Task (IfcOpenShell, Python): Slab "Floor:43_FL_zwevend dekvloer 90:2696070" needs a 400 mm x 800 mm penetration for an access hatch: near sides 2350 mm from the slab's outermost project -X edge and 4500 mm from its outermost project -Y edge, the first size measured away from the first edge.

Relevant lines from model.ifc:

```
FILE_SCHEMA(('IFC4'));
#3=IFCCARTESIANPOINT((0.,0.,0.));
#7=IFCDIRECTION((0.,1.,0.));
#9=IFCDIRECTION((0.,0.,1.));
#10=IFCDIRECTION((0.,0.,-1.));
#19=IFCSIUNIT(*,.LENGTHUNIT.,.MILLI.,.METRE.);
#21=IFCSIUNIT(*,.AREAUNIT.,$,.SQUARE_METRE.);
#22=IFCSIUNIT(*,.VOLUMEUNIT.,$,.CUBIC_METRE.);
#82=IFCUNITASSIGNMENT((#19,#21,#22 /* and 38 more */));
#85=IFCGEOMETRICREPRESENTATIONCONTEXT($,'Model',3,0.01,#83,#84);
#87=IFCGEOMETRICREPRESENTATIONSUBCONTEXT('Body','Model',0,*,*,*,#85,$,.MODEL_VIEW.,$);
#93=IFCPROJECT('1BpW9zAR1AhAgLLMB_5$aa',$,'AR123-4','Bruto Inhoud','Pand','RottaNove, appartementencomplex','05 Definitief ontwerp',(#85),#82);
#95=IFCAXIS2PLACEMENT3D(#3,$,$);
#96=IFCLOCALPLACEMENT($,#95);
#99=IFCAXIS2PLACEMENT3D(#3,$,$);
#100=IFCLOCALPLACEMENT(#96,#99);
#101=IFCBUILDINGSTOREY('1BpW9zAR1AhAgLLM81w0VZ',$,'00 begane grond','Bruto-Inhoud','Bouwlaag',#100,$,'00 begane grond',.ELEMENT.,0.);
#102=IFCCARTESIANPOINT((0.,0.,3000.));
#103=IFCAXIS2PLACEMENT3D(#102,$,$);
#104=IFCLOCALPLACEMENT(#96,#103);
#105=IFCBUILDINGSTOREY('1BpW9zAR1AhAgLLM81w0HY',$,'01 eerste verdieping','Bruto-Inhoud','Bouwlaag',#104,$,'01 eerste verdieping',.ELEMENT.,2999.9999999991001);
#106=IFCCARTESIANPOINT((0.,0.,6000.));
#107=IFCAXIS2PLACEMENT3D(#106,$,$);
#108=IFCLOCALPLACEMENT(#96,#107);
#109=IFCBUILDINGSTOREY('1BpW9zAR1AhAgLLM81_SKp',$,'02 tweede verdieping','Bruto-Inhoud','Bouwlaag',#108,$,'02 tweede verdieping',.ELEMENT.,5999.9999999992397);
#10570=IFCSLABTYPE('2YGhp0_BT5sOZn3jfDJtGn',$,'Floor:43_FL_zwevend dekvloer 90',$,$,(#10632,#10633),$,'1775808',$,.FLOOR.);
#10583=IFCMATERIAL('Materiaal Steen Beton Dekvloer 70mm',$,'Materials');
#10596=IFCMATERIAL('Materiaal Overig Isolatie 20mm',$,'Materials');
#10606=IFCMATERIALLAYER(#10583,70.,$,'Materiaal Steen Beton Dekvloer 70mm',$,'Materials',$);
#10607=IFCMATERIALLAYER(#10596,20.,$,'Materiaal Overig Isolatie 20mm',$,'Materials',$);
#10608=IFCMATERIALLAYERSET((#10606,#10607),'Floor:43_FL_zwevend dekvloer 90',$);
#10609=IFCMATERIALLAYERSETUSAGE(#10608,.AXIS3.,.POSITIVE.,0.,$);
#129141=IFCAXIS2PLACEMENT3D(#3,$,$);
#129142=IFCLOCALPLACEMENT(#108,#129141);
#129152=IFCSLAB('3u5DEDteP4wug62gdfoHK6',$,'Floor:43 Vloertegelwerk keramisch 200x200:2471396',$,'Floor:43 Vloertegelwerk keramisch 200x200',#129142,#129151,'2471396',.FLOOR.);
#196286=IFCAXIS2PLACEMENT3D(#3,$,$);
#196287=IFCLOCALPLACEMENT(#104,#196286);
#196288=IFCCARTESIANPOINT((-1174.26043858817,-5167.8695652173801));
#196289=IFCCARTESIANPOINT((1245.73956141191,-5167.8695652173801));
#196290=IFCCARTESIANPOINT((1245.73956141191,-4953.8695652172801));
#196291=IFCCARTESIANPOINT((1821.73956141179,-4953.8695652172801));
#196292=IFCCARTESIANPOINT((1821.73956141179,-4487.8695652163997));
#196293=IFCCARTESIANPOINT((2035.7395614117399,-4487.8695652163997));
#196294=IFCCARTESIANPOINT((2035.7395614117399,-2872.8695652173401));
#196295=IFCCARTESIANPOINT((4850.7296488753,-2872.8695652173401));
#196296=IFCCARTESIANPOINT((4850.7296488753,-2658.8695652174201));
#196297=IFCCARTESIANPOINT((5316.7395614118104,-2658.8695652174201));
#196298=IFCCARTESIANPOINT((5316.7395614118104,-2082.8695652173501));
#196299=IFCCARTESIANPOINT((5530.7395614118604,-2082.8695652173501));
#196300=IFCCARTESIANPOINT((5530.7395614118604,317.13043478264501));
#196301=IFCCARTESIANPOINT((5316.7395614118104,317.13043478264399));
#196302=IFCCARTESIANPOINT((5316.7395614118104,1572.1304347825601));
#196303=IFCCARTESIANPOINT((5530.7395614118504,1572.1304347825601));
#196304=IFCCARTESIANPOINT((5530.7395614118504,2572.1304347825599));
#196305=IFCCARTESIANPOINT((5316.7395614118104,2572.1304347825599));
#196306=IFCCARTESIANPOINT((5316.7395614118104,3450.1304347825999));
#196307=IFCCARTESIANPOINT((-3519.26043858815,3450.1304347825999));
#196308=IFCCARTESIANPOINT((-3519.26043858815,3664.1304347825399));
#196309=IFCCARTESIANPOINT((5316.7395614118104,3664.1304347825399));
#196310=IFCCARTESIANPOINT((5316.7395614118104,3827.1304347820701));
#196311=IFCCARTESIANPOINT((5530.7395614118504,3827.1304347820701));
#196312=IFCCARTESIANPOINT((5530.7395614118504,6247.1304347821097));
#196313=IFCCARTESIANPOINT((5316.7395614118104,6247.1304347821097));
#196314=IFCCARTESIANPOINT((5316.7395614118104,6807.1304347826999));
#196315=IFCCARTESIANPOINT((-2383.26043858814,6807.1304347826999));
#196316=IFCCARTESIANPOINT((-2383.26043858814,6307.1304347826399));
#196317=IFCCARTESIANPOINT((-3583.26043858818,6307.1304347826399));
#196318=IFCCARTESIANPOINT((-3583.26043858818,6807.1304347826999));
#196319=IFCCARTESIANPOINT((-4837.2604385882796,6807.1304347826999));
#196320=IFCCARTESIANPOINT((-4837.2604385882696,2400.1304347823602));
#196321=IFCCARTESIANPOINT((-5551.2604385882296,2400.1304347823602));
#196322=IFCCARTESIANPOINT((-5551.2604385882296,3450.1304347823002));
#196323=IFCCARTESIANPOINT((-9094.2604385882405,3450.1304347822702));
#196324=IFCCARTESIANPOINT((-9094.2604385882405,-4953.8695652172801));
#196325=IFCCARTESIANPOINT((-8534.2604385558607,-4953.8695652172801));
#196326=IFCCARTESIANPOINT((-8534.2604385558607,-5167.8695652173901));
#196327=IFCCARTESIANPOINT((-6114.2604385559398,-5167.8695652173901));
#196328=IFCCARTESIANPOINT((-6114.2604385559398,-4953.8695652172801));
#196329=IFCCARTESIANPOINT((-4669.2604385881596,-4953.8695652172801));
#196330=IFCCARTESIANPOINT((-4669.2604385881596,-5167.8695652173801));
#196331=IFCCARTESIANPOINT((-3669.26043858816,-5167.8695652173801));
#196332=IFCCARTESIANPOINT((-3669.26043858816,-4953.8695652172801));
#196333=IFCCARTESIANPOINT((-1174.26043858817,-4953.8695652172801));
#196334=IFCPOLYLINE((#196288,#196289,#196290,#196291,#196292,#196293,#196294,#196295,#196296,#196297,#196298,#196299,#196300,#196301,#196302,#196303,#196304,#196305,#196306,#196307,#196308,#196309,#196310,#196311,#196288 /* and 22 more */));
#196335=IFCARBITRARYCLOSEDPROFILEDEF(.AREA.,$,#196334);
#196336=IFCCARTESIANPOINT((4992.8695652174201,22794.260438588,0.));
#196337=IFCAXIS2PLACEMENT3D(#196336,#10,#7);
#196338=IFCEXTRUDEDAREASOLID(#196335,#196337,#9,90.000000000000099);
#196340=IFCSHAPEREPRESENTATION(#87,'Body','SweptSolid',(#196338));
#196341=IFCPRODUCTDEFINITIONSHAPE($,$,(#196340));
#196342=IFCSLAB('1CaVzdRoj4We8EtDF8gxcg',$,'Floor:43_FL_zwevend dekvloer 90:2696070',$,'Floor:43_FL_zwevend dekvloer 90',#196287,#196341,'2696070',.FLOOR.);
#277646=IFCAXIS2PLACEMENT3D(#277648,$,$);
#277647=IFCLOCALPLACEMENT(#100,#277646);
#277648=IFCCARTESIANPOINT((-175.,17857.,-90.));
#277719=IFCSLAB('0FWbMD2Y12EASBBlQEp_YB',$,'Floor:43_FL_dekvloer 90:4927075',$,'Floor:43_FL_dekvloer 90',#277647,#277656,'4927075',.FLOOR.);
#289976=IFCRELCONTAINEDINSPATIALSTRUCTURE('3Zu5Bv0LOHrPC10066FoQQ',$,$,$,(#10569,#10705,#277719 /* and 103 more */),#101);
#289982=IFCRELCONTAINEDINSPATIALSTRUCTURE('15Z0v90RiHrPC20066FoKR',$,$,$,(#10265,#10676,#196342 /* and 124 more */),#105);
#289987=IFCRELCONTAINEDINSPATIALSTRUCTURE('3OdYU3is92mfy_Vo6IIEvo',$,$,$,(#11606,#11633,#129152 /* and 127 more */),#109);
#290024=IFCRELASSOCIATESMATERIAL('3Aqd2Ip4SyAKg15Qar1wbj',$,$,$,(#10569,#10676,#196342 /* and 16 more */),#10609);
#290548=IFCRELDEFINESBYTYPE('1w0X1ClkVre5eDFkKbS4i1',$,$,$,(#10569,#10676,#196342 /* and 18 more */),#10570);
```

```python
import numpy as np
import ifcopenshell
import ifcopenshell.api.feature
import ifcopenshell.api.geometry
import ifcopenshell.api.root
import ifcopenshell.geom
import ifcopenshell.util.placement
import ifcopenshell.util.representation
import ifcopenshell.util.shape
import ifcopenshell.util.unit

model = ifcopenshell.open("model.ifc")
unit_scale = ifcopenshell.util.unit.calculate_unit_scale(model)
settings = ifcopenshell.geom.settings()


def volume(element):
    """Net volume in cubic metres, openings subtracted."""
    shape = ifcopenshell.geom.create_shape(settings, element)
    return ifcopenshell.util.shape.get_volume(shape.geometry)


slab = model.by_guid("1CaVzdRoj4We8EtDF8gxcg")
before = volume(slab)

# Extent in the slab's own axes, in metres. The edges named are its -X and -Y sides.
slab_shape = ifcopenshell.geom.create_shape(settings, slab)
vertices = ifcopenshell.util.shape.get_vertices(slab_shape.geometry)
x_min, y_min, bottom = vertices.min(axis=0)
top = vertices[:, 2].max()

opening = ifcopenshell.api.root.create_entity(model, ifc_class="IfcOpeningElement", name="Access hatch opening", predefined_type="OPENING")
context = ifcopenshell.util.representation.get_context(model, "Model", "Body", "MODEL_VIEW")
width, depth = 0.4, 0.8
outline = [(0.0, 0.0), (width, 0.0), (width, depth), (0.0, depth), (0.0, 0.0)]
# Overshoot both faces by 50 mm so the cut is clean.
shape = ifcopenshell.api.geometry.add_slab_representation(
    model, context=context, depth=top - bottom + 0.1, polyline=outline
)
ifcopenshell.api.geometry.assign_representation(model, product=opening, representation=shape)

matrix = ifcopenshell.util.placement.get_local_placement(slab.ObjectPlacement)
matrix[:, 3] = matrix @ np.append(np.array([x_min + 2.35, y_min + 4.5, bottom - 0.05]) / unit_scale, 1.0)
ifcopenshell.api.geometry.edit_object_placement(model, product=opening, matrix=matrix, is_si=False)
ifcopenshell.api.feature.add_feature(model, feature=opening, element=slab)

after = volume(slab)

print(f"slab volume {before:.3f} -> {after:.3f} m3")

model.write("model-out.ifc")
```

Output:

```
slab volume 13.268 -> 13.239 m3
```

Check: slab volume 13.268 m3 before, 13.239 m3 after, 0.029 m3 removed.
